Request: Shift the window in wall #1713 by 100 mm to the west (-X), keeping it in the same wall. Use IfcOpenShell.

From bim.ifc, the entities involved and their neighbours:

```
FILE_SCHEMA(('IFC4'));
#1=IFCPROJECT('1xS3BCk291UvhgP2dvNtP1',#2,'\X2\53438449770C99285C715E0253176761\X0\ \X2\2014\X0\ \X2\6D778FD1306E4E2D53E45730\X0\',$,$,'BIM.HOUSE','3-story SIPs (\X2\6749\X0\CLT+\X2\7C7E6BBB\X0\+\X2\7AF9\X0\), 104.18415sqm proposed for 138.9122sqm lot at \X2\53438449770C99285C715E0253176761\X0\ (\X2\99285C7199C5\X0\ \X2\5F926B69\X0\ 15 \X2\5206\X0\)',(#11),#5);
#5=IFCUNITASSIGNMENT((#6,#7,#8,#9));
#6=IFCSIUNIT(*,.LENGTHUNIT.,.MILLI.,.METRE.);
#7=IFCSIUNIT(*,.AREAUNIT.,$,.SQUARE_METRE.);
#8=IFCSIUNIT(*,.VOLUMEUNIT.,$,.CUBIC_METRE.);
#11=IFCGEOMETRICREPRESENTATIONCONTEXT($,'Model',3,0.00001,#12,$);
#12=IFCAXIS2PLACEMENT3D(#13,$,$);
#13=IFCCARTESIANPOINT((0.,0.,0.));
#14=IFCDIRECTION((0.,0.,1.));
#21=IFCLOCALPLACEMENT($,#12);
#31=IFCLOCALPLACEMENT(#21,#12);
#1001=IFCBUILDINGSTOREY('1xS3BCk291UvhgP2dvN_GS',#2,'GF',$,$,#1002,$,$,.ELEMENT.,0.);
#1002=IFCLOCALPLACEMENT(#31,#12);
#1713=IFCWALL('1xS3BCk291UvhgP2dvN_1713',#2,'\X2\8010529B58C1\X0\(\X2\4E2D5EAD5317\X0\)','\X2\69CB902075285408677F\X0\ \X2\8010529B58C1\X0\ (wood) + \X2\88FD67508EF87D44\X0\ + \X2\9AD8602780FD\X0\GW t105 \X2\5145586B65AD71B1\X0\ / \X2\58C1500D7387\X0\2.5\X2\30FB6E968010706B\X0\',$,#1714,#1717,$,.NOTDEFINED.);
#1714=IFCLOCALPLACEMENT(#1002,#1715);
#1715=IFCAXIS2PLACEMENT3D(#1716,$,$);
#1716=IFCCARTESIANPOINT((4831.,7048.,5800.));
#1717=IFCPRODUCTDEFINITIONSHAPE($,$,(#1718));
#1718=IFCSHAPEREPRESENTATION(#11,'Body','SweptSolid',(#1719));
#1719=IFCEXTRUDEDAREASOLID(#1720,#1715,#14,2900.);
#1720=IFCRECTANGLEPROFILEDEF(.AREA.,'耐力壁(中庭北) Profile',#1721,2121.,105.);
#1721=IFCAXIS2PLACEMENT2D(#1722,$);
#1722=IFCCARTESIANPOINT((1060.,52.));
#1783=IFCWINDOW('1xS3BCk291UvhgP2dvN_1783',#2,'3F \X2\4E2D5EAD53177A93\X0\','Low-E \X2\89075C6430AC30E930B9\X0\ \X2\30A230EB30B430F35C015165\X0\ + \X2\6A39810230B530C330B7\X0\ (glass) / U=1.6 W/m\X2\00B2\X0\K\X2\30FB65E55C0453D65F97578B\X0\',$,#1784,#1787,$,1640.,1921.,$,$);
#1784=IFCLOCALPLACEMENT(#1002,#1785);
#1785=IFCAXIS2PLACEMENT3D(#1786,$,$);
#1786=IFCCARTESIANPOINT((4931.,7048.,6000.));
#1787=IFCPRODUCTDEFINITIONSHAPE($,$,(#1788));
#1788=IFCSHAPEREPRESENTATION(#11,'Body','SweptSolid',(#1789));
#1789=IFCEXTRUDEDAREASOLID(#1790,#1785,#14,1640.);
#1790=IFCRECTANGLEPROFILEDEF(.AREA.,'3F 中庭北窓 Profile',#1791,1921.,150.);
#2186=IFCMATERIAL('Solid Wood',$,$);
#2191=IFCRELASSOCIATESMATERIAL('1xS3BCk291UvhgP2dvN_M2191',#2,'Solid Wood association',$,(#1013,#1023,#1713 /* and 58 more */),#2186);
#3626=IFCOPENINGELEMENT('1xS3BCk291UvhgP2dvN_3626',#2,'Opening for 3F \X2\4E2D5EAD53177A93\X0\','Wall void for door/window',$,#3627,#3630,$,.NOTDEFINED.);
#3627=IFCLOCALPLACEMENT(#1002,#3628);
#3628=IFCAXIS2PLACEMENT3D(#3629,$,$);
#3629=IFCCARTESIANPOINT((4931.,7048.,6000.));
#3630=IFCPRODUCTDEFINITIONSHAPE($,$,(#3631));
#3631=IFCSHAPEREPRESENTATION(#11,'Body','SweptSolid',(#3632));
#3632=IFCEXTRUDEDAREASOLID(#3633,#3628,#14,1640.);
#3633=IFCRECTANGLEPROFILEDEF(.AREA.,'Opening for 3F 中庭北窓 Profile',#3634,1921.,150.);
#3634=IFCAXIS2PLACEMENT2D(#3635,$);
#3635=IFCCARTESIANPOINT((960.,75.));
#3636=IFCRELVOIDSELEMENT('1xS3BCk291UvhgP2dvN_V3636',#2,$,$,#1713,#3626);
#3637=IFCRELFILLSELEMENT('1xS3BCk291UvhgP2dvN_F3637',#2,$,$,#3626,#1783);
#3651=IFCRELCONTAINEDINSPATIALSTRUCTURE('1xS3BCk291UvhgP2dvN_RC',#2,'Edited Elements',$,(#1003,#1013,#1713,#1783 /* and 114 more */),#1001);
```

```python
import ifcopenshell
import ifcopenshell.api.geometry
import ifcopenshell.util.placement
import ifcopenshell.util.unit

model = ifcopenshell.open("bim.ifc")
unit_scale = ifcopenshell.util.unit.calculate_unit_scale(model)

window = model.by_id(1783)
opening = window.FillsVoids[0].RelatingOpeningElement
wall = opening.VoidsElements[0].RelatingBuildingElement

wall_matrix = ifcopenshell.util.placement.get_local_placement(wall.ObjectPlacement)
shift = wall_matrix[:3, 0] * -0.1 / unit_scale
before = ifcopenshell.util.placement.get_local_placement(window.ObjectPlacement)[:3, 3].copy()

# The window is not placed relative to its opening, so move both.
for product in (opening, window):
    matrix = ifcopenshell.util.placement.get_local_placement(product.ObjectPlacement)
    matrix[:3, 3] += shift
    ifcopenshell.api.geometry.edit_object_placement(model, product=product, matrix=matrix, is_si=False)

after = ifcopenshell.util.placement.get_local_placement(window.ObjectPlacement)[:3, 3]
print("window moved by", (after - before).round(3) + 0.0)

model.write("bim_v2.ifc")
```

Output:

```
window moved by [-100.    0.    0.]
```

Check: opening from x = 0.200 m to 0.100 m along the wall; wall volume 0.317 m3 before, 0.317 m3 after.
